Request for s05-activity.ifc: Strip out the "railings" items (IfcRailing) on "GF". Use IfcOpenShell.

First a look at what the model holds.

```python
import ifcopenshell
import ifcopenshell.util.element

model = ifcopenshell.open("s05-activity.ifc")
print(model.schema)
storey = next(s for s in model.by_type("IfcBuildingStorey") if s.Name == "GF")
railings = [e for e in ifcopenshell.util.element.get_decomposition(storey) if e.is_a("IfcRailing")]
seen = {}
for e in railings:
    element_type = ifcopenshell.util.element.get_type(e)
    name = element_type.Name if element_type not in (None, e) else None
    seen[name] = seen.get(name, 0) + 1
for name, count in sorted(seen.items(), key=str):
    print(count, "x", name)
```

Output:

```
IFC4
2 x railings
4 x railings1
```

```python
import ifcopenshell
import ifcopenshell.api.root
import ifcopenshell.util.element

model = ifcopenshell.open("s05-activity.ifc")

storey = next(s for s in model.by_type("IfcBuildingStorey") if s.Name == "GF")
railings = [e for e in ifcopenshell.util.element.get_decomposition(storey) if e.is_a("IfcRailing")]
targets = [e for e in railings if (t := ifcopenshell.util.element.get_type(e)) not in (None, e) and t.Name == "railings"]

for e in targets:
    ifcopenshell.api.root.remove_product(model, product=e)
print(len(targets), "removed")

model.write("s05-activity-out.ifc")
```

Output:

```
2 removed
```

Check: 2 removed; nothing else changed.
